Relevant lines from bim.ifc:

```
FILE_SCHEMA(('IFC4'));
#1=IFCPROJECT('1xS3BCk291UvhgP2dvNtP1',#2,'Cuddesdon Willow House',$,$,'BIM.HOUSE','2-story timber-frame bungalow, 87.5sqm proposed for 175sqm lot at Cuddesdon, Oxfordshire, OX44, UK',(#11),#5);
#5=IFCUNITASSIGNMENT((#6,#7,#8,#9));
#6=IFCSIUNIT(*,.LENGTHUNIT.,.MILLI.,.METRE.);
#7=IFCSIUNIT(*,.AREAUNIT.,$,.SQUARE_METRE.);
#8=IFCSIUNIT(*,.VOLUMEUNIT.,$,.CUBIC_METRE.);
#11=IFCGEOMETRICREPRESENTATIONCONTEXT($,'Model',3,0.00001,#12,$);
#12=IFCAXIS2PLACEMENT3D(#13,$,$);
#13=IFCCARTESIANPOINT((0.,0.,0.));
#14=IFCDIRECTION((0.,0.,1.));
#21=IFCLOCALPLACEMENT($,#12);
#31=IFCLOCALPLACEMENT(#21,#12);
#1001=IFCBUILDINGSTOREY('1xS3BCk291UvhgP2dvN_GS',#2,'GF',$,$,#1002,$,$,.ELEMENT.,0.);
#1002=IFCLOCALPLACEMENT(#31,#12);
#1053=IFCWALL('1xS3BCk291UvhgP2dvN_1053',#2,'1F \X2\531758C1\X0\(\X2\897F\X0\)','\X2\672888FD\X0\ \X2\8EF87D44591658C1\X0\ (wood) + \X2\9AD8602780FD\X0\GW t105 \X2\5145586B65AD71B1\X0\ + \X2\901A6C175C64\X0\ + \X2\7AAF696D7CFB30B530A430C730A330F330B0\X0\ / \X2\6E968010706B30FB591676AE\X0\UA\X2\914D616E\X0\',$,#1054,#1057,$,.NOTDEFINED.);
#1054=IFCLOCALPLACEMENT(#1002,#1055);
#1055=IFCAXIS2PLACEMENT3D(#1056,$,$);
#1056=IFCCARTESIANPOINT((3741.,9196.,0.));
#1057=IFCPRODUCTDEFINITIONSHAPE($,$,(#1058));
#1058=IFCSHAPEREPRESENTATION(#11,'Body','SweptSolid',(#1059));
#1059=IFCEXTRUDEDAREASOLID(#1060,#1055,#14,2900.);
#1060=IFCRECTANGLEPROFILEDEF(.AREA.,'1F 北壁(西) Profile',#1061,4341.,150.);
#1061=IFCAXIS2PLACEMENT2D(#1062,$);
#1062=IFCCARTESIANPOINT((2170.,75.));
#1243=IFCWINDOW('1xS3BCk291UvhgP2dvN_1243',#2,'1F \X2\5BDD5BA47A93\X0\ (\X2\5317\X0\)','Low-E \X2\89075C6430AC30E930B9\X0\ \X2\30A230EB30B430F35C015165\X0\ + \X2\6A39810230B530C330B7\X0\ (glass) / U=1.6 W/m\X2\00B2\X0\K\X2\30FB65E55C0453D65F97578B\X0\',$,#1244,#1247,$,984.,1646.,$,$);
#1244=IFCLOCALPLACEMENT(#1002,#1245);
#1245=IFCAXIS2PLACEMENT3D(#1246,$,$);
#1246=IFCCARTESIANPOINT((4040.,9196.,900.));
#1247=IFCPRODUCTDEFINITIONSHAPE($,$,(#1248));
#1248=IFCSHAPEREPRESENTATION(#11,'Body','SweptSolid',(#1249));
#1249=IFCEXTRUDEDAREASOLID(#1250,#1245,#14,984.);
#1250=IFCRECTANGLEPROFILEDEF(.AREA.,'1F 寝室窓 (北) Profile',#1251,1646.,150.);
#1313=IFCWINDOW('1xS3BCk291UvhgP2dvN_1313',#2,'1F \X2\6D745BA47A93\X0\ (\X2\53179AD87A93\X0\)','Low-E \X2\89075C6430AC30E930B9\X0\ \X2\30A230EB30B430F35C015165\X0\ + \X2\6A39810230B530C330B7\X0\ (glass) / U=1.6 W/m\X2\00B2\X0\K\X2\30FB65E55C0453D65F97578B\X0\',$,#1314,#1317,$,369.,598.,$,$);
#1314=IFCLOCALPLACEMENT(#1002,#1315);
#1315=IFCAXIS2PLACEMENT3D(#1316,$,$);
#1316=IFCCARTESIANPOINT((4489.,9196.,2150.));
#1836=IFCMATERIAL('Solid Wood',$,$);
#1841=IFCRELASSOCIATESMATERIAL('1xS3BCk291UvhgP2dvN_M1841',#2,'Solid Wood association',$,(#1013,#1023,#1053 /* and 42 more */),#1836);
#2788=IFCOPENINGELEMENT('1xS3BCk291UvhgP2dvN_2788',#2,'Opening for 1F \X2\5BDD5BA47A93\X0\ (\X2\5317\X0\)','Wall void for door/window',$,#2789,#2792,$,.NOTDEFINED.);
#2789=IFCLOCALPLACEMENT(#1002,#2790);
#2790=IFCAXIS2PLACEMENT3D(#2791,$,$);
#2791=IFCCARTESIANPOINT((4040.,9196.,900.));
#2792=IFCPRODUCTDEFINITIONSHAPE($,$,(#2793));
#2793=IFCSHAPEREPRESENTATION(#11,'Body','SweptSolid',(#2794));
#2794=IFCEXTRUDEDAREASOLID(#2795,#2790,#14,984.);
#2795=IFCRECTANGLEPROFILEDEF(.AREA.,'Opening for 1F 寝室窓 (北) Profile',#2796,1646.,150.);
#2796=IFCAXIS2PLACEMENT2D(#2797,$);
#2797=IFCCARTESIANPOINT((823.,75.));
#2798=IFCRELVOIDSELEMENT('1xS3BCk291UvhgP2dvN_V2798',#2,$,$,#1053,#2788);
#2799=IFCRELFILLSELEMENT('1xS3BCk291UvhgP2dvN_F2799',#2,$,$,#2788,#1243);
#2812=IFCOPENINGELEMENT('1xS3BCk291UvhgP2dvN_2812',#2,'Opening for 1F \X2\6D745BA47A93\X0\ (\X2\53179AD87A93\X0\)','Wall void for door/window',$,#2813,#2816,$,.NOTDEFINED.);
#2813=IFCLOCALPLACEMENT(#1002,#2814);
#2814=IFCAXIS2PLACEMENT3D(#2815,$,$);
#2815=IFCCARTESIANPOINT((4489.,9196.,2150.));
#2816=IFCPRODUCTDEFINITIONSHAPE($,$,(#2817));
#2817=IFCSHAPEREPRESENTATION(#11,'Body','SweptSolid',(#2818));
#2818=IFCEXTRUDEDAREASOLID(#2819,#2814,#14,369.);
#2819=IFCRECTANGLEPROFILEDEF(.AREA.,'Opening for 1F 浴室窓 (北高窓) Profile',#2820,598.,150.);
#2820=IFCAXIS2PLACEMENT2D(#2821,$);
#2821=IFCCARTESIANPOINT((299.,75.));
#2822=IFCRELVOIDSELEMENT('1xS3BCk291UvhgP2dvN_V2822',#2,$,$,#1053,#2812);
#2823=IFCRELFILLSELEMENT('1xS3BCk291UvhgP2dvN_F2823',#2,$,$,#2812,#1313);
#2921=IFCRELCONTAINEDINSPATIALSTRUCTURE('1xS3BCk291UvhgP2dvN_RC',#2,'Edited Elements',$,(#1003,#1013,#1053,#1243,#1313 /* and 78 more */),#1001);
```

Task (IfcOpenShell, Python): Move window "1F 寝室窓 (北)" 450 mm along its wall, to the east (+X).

```python
import ifcopenshell
import ifcopenshell.api.geometry
import ifcopenshell.util.placement
import ifcopenshell.util.unit

model = ifcopenshell.open("bim.ifc")
unit_scale = ifcopenshell.util.unit.calculate_unit_scale(model)

window = model.by_guid("1xS3BCk291UvhgP2dvN_1243")
opening = window.FillsVoids[0].RelatingOpeningElement
wall = opening.VoidsElements[0].RelatingBuildingElement

wall_matrix = ifcopenshell.util.placement.get_local_placement(wall.ObjectPlacement)
shift = wall_matrix[:3, 0] * 0.45 / unit_scale
before = ifcopenshell.util.placement.get_local_placement(window.ObjectPlacement)[:3, 3].copy()

# The window is not placed relative to its opening, so move both.
for product in (opening, window):
    matrix = ifcopenshell.util.placement.get_local_placement(product.ObjectPlacement)
    matrix[:3, 3] += shift
    ifcopenshell.api.geometry.edit_object_placement(model, product=product, matrix=matrix, is_si=False)

after = ifcopenshell.util.placement.get_local_placement(window.ObjectPlacement)[:3, 3]
print("window moved by", (after - before).round(3) + 0.0)

model.write("bim_rev.ifc")
```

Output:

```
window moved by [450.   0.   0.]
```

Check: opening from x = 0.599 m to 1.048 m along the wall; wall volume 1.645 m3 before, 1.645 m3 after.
